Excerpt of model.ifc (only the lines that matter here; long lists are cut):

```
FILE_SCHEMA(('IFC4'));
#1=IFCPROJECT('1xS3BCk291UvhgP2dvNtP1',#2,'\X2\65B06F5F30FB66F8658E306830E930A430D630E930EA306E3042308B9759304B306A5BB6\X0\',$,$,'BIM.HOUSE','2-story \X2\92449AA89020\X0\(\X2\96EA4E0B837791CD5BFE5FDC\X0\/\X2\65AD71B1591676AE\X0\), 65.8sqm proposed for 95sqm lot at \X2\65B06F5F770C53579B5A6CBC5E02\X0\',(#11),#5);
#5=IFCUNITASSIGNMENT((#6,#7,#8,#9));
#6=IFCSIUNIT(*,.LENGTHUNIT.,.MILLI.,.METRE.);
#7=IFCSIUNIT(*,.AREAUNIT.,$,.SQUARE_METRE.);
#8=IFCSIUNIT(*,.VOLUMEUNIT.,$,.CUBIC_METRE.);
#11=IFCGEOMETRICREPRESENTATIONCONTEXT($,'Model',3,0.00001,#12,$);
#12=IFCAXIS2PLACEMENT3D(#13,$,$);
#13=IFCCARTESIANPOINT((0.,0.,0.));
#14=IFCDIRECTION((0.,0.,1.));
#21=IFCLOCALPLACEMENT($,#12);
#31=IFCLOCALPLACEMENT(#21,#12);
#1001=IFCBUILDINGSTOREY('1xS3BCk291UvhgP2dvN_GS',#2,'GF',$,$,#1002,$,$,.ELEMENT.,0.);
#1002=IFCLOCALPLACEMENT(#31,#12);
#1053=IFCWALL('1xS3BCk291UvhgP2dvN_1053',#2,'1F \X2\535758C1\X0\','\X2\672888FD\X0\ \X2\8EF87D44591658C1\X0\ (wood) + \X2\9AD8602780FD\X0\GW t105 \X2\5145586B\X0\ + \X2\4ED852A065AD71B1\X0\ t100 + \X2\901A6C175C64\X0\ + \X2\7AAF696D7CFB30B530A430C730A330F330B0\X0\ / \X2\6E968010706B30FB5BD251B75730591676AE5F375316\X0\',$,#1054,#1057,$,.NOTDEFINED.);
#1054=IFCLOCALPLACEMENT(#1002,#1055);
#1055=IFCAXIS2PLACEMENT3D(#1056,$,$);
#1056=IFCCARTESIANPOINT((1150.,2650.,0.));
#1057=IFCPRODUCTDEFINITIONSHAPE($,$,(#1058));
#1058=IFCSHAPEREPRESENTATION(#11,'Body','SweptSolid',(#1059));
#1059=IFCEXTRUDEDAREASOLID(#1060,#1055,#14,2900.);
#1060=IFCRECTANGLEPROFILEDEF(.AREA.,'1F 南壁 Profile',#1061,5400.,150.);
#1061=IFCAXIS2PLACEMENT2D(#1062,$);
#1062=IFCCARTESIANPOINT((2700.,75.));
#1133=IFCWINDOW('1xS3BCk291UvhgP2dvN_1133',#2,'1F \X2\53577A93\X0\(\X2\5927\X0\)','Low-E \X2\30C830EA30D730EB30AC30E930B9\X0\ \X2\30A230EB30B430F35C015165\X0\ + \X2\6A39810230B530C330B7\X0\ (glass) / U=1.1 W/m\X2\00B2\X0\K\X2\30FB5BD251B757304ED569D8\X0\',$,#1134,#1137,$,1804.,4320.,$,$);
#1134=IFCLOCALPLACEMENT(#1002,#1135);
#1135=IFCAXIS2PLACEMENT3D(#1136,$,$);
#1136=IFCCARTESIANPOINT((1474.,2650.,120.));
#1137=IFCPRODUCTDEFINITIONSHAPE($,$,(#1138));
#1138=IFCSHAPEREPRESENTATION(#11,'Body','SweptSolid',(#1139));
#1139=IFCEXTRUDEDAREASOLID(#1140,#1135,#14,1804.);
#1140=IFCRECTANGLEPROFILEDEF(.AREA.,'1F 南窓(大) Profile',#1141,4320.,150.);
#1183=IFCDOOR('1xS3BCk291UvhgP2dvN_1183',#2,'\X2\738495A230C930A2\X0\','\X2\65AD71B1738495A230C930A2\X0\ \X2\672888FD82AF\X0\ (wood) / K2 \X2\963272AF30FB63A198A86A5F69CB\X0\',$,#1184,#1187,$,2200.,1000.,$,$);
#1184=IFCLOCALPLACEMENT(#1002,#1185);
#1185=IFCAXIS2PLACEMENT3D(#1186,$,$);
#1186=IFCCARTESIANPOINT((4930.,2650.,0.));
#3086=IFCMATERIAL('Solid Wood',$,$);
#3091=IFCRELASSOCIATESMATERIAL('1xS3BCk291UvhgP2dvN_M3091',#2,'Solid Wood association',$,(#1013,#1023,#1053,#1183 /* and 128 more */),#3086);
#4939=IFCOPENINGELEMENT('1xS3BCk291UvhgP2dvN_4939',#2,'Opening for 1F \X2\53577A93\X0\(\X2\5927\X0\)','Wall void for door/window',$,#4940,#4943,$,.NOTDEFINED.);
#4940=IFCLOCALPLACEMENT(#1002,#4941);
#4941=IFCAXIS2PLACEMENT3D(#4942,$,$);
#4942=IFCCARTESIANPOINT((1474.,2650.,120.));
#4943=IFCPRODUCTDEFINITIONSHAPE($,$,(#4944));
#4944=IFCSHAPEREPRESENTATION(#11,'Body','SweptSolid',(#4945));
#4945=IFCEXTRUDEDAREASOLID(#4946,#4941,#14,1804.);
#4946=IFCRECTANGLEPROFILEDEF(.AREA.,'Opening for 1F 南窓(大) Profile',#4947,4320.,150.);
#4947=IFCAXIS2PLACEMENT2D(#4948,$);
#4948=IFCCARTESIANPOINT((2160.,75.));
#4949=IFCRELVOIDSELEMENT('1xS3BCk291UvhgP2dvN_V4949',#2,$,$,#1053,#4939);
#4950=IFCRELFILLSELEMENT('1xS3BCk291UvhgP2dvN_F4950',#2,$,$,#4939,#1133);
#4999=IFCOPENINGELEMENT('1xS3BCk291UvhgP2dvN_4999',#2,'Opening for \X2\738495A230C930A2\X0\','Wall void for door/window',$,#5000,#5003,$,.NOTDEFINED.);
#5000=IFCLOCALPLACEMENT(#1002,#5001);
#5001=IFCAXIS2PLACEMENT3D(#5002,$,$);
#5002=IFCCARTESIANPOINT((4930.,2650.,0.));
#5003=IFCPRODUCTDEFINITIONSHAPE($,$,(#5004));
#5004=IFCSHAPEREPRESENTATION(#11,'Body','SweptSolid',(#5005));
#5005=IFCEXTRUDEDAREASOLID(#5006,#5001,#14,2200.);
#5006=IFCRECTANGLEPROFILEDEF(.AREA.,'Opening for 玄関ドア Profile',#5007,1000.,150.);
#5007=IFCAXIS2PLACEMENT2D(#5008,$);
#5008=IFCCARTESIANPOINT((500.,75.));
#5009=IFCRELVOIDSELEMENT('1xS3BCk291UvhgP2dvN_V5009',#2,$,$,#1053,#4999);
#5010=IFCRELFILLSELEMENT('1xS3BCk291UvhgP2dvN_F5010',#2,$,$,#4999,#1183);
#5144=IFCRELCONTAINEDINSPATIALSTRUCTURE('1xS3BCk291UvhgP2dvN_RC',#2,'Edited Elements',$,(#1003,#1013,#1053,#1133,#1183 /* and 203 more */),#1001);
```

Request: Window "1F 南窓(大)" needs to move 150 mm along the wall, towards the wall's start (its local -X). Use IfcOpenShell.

```python
import ifcopenshell
import ifcopenshell.api.geometry
import ifcopenshell.util.placement
import ifcopenshell.util.unit

model = ifcopenshell.open("model.ifc")
unit_scale = ifcopenshell.util.unit.calculate_unit_scale(model)

window = model.by_id(1133)
opening = window.FillsVoids[0].RelatingOpeningElement
wall = opening.VoidsElements[0].RelatingBuildingElement

wall_matrix = ifcopenshell.util.placement.get_local_placement(wall.ObjectPlacement)
shift = wall_matrix[:3, 0] * -0.15 / unit_scale
before = ifcopenshell.util.placement.get_local_placement(window.ObjectPlacement)[:3, 3].copy()

# The window is not placed relative to its opening, so move both.
for product in (opening, window):
    matrix = ifcopenshell.util.placement.get_local_placement(product.ObjectPlacement)
    matrix[:3, 3] += shift
    ifcopenshell.api.geometry.edit_object_placement(model, product=product, matrix=matrix, is_si=False)

after = ifcopenshell.util.placement.get_local_placement(window.ObjectPlacement)[:3, 3]
print("window moved by", (after - before).round(3) + 0.0)

model.write("model_edited.ifc")
```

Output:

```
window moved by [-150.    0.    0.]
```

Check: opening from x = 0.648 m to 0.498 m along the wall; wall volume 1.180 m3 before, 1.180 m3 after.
